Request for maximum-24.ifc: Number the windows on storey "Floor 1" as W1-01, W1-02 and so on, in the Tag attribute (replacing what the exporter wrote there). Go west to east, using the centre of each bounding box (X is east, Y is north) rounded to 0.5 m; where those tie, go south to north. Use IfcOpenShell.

First a look at what the model holds.

```python
import ifcopenshell
import ifcopenshell.util.element
import ifcopenshell.util.placement

model = ifcopenshell.open("maximum-24.ifc")
print(model.schema)
storey = next(s for s in model.by_type("IfcBuildingStorey") if s.Name == "Floor 1")
windows = [e for e in ifcopenshell.util.element.get_decomposition(storey) if e.is_a("IfcWindow")]
for e in sorted(windows, key=lambda e: e.id()):
    origin = ifcopenshell.util.placement.get_local_placement(e.ObjectPlacement)[:3, 3]
    print(e.id(), e.Tag, e.Name, origin.round(2) + 0.0, sep=" | ")
```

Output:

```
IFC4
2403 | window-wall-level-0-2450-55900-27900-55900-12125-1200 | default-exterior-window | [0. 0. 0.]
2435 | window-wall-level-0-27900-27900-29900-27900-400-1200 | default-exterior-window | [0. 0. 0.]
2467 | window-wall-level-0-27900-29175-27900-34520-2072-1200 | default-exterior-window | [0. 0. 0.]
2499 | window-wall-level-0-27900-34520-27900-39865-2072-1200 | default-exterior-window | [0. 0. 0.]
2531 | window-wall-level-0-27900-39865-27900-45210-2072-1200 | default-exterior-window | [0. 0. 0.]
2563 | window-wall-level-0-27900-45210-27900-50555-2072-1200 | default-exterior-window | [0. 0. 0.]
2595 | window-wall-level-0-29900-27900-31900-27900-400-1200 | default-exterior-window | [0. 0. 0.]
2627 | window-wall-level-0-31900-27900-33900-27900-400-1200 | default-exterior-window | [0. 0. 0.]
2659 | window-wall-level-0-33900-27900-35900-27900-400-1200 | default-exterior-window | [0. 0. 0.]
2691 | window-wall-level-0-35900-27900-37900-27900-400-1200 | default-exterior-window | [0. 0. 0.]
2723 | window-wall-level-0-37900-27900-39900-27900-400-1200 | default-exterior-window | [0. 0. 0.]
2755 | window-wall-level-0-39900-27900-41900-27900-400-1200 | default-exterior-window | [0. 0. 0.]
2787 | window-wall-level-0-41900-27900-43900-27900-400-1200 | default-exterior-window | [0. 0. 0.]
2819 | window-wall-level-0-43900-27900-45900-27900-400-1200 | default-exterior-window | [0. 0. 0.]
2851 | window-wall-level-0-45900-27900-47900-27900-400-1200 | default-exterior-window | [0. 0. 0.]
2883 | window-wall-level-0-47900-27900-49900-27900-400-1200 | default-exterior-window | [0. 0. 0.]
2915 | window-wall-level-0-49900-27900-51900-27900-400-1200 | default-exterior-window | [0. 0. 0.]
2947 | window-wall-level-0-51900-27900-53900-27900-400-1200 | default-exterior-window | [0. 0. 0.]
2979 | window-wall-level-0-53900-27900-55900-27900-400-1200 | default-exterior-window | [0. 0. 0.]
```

```python
import ifcopenshell
import ifcopenshell.geom
import ifcopenshell.util.element
import ifcopenshell.util.shape

model = ifcopenshell.open("maximum-24.ifc")
settings = ifcopenshell.geom.settings()
settings.set("use-world-coords", True)


def centre(element):
    shape = ifcopenshell.geom.create_shape(settings, element)
    return ifcopenshell.util.shape.get_bbox_centroid(shape.geometry)


storey = next(s for s in model.by_type("IfcBuildingStorey") if s.Name == "Floor 1")
windows = [e for e in ifcopenshell.util.element.get_decomposition(storey) if e.is_a("IfcWindow")]

# Insertion points can sit at a corner or the storey origin, so sort by the geometry (in metres).
centres = {e: centre(e) for e in windows}
windows.sort(key=lambda e: (round(centres[e][0] / 0.5), centres[e][1]))

for i, e in enumerate(windows, start=1):
    number = f"W1-{i:02d}"
    e.Tag = number
    print(e.id(), number)

model.write("maximum-24-out.ifc")
```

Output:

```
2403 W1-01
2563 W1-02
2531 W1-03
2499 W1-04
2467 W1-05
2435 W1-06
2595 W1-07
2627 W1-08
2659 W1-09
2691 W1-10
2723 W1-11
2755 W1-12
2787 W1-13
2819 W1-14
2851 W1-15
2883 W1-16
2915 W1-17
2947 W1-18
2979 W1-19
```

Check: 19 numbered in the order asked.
